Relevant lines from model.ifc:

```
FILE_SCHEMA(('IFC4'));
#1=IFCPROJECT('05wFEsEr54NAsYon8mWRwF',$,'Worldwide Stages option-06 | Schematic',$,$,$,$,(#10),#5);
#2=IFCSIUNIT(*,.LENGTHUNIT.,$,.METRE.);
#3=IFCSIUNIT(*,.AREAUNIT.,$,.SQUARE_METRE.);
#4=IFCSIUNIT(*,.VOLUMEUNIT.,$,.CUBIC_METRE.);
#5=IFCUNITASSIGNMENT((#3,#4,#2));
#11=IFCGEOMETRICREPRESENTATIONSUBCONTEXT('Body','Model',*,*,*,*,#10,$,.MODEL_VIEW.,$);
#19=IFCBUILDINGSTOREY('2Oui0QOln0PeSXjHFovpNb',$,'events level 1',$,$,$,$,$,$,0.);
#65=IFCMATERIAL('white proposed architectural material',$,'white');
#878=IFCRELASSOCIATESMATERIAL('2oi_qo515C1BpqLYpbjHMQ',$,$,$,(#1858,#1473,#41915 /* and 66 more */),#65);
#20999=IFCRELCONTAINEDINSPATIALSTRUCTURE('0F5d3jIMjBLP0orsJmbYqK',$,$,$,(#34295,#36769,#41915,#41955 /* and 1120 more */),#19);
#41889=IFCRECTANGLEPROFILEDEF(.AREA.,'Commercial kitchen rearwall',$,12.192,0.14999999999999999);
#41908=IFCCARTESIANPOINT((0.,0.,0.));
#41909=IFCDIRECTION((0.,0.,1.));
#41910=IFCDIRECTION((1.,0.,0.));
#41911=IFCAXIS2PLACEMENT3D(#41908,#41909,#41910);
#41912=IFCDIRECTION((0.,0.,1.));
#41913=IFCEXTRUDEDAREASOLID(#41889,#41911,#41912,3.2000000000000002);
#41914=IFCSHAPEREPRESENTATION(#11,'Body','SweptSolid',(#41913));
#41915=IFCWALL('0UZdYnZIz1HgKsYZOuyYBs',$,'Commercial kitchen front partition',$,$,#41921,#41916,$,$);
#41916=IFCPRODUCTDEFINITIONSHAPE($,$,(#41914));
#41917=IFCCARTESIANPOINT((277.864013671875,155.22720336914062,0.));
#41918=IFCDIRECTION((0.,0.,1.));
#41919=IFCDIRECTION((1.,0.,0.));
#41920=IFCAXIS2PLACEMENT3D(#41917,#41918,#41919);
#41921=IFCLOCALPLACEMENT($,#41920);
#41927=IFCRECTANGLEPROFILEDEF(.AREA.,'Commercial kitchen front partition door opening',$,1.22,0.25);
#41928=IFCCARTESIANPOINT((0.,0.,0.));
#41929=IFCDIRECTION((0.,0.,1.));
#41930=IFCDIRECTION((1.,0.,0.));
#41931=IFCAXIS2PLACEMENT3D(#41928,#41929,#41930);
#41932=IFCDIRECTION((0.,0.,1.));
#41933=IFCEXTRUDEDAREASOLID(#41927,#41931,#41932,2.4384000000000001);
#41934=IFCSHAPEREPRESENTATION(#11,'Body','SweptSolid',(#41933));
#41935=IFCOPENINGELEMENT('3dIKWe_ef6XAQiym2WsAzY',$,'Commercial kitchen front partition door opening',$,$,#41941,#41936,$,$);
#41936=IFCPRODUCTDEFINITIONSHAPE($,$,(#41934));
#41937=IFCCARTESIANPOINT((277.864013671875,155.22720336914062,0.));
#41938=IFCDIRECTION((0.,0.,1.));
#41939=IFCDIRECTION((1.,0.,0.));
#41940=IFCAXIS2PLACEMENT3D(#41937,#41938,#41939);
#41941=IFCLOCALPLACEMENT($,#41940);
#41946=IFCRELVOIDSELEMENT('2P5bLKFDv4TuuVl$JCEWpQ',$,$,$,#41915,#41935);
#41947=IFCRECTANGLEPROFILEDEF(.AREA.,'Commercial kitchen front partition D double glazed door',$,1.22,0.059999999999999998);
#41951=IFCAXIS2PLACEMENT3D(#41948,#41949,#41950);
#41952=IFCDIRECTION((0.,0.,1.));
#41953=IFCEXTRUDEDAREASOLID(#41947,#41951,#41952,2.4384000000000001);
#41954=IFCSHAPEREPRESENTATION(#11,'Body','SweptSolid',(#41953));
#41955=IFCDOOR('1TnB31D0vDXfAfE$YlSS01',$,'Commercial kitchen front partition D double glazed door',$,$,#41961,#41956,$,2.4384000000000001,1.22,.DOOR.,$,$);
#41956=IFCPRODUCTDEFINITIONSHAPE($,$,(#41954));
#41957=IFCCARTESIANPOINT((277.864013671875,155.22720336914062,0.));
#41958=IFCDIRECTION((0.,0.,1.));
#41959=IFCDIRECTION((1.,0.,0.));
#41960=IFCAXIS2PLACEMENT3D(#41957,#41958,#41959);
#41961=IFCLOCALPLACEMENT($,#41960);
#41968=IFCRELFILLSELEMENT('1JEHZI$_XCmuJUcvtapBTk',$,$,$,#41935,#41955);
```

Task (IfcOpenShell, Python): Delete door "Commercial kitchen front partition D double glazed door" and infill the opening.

```python
import ifcopenshell
import ifcopenshell.api.feature
import ifcopenshell.api.root
import ifcopenshell.geom
import ifcopenshell.util.shape

model = ifcopenshell.open("model.ifc")
settings = ifcopenshell.geom.settings()


def volume(element):
    """Net volume in cubic metres, openings subtracted."""
    shape = ifcopenshell.geom.create_shape(settings, element)
    return ifcopenshell.util.shape.get_volume(shape.geometry)


door = model.by_guid("1TnB31D0vDXfAfE$YlSS01")
opening = door.FillsVoids[0].RelatingOpeningElement
wall = opening.VoidsElements[0].RelatingBuildingElement
before = volume(wall)

ifcopenshell.api.root.remove_product(model, product=door)
ifcopenshell.api.feature.remove_feature(model, feature=opening)

after = volume(wall)

print(f"wall volume {before:.3f} -> {after:.3f} m3")

model.write("model_v2.ifc")
```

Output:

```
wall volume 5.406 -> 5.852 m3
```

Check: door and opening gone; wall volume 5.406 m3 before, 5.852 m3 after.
